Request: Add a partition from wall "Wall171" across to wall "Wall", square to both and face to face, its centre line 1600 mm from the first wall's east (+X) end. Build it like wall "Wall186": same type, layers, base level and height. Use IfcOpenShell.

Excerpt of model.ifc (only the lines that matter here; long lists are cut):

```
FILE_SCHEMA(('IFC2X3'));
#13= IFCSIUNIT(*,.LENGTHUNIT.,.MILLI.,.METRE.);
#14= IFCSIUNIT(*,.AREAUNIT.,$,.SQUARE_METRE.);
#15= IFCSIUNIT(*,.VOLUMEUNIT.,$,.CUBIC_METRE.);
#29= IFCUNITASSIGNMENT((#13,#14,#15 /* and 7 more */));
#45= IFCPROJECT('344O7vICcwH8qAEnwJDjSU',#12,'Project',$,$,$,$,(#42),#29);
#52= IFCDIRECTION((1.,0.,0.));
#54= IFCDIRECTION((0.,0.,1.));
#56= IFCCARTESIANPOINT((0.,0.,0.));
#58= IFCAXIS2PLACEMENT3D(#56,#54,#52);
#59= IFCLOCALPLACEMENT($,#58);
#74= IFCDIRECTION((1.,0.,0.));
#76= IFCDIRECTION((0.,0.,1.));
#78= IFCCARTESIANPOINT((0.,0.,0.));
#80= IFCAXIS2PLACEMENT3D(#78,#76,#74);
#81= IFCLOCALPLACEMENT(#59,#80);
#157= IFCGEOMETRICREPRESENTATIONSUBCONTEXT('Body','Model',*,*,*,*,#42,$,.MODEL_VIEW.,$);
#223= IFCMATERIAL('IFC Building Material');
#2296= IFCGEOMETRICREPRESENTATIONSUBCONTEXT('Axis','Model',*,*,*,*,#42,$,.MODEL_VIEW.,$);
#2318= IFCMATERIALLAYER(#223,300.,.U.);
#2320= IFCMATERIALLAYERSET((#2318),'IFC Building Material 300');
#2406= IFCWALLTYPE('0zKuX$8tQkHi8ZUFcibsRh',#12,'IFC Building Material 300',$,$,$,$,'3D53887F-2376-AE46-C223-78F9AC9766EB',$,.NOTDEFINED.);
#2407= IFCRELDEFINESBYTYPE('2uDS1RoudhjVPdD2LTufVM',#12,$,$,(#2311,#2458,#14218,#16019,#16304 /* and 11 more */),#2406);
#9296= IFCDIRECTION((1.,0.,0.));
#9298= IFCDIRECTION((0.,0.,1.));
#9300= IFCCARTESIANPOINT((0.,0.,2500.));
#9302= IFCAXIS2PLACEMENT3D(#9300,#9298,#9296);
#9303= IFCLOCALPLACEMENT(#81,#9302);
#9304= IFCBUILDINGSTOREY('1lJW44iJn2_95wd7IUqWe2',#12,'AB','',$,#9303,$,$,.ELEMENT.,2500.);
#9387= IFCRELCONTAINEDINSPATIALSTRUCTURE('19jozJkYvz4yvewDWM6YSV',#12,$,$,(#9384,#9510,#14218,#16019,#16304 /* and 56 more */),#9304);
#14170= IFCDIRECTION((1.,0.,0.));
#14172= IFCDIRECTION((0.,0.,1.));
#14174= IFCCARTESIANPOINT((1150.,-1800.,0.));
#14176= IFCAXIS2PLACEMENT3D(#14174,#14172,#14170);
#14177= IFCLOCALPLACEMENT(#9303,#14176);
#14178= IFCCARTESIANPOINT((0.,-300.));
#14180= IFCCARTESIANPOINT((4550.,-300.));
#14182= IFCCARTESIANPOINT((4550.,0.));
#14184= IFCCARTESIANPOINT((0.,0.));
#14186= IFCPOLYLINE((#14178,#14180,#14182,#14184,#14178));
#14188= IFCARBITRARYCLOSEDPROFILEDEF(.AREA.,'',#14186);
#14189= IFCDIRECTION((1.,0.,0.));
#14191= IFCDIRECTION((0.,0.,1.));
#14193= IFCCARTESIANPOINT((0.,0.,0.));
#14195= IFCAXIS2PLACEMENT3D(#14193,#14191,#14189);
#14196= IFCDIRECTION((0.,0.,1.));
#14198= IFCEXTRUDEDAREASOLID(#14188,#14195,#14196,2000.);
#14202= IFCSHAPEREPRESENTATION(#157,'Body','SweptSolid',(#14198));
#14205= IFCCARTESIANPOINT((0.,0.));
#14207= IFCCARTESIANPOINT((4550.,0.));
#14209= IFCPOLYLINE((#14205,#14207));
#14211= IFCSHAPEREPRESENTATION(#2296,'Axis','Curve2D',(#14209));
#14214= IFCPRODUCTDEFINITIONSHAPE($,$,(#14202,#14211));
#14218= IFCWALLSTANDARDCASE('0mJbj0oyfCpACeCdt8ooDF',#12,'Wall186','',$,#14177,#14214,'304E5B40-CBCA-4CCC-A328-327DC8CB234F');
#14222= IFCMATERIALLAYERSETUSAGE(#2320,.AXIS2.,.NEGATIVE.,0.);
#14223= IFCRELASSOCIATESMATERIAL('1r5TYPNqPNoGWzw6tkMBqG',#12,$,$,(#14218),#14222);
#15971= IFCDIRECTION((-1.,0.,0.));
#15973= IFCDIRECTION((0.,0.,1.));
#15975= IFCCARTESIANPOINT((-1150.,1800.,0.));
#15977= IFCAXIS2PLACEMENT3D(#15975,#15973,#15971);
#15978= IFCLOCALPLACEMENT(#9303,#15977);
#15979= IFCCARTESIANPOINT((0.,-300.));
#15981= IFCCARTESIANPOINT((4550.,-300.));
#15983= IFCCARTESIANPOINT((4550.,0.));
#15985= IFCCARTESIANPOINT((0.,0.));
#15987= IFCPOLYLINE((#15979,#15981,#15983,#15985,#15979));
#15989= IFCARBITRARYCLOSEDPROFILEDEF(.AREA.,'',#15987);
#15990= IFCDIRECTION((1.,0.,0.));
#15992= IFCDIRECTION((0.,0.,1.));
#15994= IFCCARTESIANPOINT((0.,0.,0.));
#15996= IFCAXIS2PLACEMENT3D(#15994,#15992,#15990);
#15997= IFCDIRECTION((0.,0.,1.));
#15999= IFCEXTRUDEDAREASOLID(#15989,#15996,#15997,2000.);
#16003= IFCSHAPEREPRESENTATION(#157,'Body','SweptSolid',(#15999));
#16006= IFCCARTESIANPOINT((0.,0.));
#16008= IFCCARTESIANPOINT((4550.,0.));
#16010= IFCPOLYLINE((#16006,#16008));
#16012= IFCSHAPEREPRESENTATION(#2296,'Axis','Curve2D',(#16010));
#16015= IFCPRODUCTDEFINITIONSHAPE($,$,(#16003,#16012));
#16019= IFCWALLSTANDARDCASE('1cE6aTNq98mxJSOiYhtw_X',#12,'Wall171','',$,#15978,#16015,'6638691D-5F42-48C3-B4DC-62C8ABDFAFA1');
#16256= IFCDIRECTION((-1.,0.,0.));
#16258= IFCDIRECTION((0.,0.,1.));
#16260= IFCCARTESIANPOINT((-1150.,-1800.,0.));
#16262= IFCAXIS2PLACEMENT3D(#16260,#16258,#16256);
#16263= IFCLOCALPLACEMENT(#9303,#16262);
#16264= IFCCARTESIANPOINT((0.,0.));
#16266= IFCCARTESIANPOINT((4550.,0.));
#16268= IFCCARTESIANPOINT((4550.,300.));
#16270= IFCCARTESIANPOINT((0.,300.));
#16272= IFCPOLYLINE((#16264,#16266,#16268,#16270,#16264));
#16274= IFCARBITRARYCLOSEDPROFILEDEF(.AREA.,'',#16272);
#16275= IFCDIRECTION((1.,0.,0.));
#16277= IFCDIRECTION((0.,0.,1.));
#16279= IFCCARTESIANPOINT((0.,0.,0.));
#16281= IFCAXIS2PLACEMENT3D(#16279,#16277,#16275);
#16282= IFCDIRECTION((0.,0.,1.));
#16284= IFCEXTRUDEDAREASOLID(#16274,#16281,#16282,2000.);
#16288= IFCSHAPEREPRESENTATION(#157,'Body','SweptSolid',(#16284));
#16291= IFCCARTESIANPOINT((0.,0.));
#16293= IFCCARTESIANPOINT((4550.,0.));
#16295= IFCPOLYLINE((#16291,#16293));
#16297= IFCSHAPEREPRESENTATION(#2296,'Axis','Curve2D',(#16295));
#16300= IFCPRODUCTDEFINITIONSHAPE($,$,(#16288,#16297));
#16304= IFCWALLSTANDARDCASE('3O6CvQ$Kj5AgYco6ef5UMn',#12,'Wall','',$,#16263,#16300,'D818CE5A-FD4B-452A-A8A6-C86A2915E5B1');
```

```python
import numpy as np
import ifcopenshell
import ifcopenshell.api.geometry
import ifcopenshell.api.material
import ifcopenshell.api.pset
import ifcopenshell.api.root
import ifcopenshell.api.spatial
import ifcopenshell.api.type
import ifcopenshell.geom
import ifcopenshell.util.element
import ifcopenshell.util.placement
import ifcopenshell.util.representation
import ifcopenshell.util.shape
import ifcopenshell.util.unit

model = ifcopenshell.open("model.ifc")
unit_scale = ifcopenshell.util.unit.calculate_unit_scale(model)
settings = ifcopenshell.geom.settings()
settings.set("use-world-coords", True)

start_wall = model.by_guid("1cE6aTNq98mxJSOiYhtw_X")
end_wall = model.by_guid("3O6CvQ$Kj5AgYco6ef5UMn")
like = model.by_id(14218)
matrix = ifcopenshell.util.placement.get_local_placement(start_wall.ObjectPlacement)
matrix[:3, 3] *= unit_scale


def extent(element):
    """Bounding box in the first wall's axes, in metres."""
    shape = ifcopenshell.geom.create_shape(settings, element)
    points = (ifcopenshell.util.shape.get_vertices(shape.geometry) - matrix[:3, 3]) @ matrix[:3, :3]
    return points.min(axis=0), points.max(axis=0)


y_start = extent(start_wall)[1][1]
y_end = extent(end_wall)[0][1]
like_min, like_max = extent(like)
length, height = float(abs(y_end - y_start)), float(like_max[2] - like_min[2])
layer_set = ifcopenshell.util.element.get_material(like, should_skip_usage=True)
thickness = sum(layer.LayerThickness for layer in layer_set.MaterialLayers) * unit_scale

wall = ifcopenshell.api.root.create_entity(model, ifc_class="IfcWallStandardCase", name="New partition")
storey = ifcopenshell.util.element.get_container(like)
ifcopenshell.api.spatial.assign_container(model, products=[wall], relating_structure=storey)
ifcopenshell.api.type.assign_type(
    model, related_objects=[wall], relating_type=ifcopenshell.util.element.get_type(like), should_map_representations=False
)
rel = ifcopenshell.api.material.assign_material(
    model, products=[wall], type="IfcMaterialLayerSetUsage", material=layer_set
)
rel.RelatingMaterial.OffsetFromReferenceLine = -thickness / 2 / unit_scale
pset = ifcopenshell.api.pset.add_pset(model, product=wall, name="Pset_WallCommon")
ifcopenshell.api.pset.edit_pset(model, pset=pset, properties={"IsExternal": False, "LoadBearing": False})

# The axis runs down the middle of the wall.
axis = ifcopenshell.api.geometry.add_axis_representation(
    model, context=ifcopenshell.util.representation.get_context(model, "Model", "Axis"), axis=[(0.0, 0.0), (length, 0.0)]
)
body = ifcopenshell.api.geometry.add_wall_representation(
    model,
    context=ifcopenshell.util.representation.get_context(model, "Model", "Body", "MODEL_VIEW"),
    length=length,
    height=height,
    thickness=thickness,
    offset=-thickness / 2,
)
for representation in (axis, body):
    ifcopenshell.api.geometry.assign_representation(model, product=wall, representation=representation)

placement = matrix @ ifcopenshell.util.placement.rotation(90, "Z")
placement[:, 3] = matrix @ np.array([extent(start_wall)[0][0] + 1.6, y_start, like_min[2], 1.0])
ifcopenshell.api.geometry.edit_object_placement(model, product=wall, matrix=placement)

print(f"partition {length:.3f} m long, {height:.3f} m high, {thickness:.3f} m thick")

model.write("model_edited.ifc")
```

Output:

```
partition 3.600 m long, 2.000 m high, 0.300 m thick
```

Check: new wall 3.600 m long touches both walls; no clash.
